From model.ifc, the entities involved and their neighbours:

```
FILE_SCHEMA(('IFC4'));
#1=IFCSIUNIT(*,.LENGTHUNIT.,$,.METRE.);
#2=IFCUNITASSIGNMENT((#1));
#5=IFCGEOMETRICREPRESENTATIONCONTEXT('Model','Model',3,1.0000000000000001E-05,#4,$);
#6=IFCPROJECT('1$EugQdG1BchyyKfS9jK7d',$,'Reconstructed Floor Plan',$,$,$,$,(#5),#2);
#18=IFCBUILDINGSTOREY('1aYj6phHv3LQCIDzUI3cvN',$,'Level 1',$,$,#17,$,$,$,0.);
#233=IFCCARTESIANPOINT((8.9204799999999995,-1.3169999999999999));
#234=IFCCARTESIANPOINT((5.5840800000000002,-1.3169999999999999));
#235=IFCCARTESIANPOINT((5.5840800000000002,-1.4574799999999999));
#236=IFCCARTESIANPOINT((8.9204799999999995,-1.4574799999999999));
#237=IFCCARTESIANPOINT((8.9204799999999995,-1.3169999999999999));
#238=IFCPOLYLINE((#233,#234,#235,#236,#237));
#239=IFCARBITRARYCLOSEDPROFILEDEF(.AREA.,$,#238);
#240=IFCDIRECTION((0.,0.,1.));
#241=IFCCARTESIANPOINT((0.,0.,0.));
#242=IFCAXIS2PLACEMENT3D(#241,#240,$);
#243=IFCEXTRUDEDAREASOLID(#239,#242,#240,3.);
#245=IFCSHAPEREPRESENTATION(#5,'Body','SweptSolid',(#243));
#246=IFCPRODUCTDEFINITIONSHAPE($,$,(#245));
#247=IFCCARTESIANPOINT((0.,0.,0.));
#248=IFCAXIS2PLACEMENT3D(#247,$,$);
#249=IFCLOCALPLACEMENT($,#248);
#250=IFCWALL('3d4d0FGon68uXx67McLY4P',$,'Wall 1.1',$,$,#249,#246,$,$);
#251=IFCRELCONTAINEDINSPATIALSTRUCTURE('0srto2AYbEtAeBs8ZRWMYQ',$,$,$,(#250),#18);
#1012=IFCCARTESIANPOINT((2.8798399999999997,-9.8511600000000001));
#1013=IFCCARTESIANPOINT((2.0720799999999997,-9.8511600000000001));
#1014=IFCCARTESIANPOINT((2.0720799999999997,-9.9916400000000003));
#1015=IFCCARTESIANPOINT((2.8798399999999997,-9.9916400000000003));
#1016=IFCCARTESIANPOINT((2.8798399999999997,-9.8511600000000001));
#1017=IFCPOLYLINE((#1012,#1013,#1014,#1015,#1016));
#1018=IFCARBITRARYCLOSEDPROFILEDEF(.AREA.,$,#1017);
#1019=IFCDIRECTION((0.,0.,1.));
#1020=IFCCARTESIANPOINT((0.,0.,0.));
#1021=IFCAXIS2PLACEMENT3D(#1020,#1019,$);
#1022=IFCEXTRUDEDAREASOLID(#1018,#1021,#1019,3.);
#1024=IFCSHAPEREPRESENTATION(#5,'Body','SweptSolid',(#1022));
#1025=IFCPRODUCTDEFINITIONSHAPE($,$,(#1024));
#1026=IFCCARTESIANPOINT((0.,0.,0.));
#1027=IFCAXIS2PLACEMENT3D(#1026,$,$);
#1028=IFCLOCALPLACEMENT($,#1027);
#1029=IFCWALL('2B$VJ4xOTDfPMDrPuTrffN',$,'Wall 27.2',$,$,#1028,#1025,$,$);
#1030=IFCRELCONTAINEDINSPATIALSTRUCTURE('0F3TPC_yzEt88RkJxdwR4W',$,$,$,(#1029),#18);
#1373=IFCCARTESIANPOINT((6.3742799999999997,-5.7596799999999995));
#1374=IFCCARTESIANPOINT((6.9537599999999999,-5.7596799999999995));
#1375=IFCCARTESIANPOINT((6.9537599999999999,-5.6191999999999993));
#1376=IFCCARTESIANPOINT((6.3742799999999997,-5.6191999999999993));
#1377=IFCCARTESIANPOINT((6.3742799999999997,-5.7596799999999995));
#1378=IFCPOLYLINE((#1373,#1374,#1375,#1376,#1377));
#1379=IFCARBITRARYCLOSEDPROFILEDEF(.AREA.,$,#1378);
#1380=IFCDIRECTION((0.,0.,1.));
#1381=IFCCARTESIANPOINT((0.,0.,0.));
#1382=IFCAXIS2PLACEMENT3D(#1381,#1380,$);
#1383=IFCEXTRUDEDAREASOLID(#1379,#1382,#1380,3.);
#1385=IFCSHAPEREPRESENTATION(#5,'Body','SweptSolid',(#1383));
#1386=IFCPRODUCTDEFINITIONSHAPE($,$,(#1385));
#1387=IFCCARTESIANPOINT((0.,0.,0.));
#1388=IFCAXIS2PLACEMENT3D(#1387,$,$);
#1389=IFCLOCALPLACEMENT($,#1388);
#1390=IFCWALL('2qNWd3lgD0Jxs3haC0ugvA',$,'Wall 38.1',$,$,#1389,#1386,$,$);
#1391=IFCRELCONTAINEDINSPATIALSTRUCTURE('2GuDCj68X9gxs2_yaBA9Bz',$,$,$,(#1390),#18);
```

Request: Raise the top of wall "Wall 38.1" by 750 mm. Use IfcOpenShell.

```python
import ifcopenshell
import ifcopenshell.geom
import ifcopenshell.util.shape
import ifcopenshell.util.unit

model = ifcopenshell.open("model.ifc")
unit_scale = ifcopenshell.util.unit.calculate_unit_scale(model)
settings = ifcopenshell.geom.settings()


def volume(element):
    """Net volume in cubic metres, openings subtracted."""
    shape = ifcopenshell.geom.create_shape(settings, element)
    return ifcopenshell.util.shape.get_volume(shape.geometry)


wall = model.by_guid("2qNWd3lgD0Jxs3haC0ugvA")
before = volume(wall)

body = next(r for r in wall.Representation.Representations if r.RepresentationIdentifier == "Body")
solid = body.Items[0]
old_height = solid.Depth
solid.Depth += 0.75 / unit_scale
after = volume(wall)

print(f"height {old_height:g} -> {solid.Depth:g}, volume {before:.3f} -> {after:.3f} m3")

model.write("model_updated.ifc")
```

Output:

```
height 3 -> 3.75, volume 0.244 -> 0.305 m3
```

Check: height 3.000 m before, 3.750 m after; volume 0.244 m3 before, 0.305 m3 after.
